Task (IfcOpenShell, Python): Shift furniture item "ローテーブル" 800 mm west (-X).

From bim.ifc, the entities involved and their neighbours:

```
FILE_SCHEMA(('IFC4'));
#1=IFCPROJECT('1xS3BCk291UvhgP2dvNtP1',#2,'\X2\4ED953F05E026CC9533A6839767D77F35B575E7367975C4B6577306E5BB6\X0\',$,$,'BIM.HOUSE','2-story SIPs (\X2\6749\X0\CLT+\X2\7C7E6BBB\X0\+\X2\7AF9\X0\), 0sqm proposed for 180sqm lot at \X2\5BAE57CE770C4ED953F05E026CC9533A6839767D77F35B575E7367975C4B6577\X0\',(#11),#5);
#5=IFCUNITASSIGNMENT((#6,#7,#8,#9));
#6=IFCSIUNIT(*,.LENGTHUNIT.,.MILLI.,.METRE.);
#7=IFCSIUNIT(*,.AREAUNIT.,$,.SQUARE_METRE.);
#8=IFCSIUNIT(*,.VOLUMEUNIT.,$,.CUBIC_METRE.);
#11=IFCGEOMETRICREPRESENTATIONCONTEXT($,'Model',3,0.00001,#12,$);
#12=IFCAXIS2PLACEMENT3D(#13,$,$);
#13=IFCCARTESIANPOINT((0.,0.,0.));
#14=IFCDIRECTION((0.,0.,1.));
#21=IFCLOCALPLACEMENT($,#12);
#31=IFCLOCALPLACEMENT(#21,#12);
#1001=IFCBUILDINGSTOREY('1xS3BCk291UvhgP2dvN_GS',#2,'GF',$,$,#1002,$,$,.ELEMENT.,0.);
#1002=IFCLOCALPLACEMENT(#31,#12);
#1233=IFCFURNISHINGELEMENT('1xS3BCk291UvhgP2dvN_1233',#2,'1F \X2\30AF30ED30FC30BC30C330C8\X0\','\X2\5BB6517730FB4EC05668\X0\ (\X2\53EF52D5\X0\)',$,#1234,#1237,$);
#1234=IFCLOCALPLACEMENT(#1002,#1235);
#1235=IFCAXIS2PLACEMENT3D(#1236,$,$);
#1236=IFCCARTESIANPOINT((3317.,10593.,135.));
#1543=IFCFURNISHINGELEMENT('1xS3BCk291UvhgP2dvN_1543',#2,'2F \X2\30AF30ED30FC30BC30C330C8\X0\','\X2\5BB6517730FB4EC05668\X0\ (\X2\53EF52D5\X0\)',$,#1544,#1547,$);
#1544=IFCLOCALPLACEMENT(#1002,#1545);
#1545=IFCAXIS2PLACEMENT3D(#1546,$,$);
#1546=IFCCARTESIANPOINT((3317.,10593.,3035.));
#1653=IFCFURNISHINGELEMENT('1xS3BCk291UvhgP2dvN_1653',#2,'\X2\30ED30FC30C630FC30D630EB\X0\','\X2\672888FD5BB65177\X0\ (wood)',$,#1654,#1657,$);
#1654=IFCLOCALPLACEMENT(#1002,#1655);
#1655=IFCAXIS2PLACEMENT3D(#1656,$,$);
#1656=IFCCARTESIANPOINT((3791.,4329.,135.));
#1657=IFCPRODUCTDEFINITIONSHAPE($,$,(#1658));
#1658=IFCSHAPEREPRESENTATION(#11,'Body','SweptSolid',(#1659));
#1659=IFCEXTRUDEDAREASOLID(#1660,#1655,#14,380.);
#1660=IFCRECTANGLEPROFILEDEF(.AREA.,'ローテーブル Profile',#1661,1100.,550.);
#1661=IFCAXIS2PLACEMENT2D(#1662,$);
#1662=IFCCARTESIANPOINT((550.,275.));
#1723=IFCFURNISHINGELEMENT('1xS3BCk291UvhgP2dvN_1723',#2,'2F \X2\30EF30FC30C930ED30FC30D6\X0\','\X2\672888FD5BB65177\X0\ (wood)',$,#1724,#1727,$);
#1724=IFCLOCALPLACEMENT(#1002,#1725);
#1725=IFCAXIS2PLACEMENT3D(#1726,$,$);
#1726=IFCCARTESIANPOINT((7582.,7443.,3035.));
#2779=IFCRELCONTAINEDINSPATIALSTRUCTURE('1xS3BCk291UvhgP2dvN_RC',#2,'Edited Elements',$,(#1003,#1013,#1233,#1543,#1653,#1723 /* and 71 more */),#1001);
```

```python
import ifcopenshell
import ifcopenshell.api.geometry
import ifcopenshell.util.placement
import ifcopenshell.util.unit

model = ifcopenshell.open("bim.ifc")
unit_scale = ifcopenshell.util.unit.calculate_unit_scale(model)

item = model.by_guid("1xS3BCk291UvhgP2dvN_1653")
matrix = ifcopenshell.util.placement.get_local_placement(item.ObjectPlacement)
matrix[0, 3] -= 0.8 / unit_scale
ifcopenshell.api.geometry.edit_object_placement(model, product=item, matrix=matrix, is_si=False)

print(ifcopenshell.util.placement.get_local_placement(item.ObjectPlacement).round(3) + 0.0)

model.write("bim_updated.ifc")
```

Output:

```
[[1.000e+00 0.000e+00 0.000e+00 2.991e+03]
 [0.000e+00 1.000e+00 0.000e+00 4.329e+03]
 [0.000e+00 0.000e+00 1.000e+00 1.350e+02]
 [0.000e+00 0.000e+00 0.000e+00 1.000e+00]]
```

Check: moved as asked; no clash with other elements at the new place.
